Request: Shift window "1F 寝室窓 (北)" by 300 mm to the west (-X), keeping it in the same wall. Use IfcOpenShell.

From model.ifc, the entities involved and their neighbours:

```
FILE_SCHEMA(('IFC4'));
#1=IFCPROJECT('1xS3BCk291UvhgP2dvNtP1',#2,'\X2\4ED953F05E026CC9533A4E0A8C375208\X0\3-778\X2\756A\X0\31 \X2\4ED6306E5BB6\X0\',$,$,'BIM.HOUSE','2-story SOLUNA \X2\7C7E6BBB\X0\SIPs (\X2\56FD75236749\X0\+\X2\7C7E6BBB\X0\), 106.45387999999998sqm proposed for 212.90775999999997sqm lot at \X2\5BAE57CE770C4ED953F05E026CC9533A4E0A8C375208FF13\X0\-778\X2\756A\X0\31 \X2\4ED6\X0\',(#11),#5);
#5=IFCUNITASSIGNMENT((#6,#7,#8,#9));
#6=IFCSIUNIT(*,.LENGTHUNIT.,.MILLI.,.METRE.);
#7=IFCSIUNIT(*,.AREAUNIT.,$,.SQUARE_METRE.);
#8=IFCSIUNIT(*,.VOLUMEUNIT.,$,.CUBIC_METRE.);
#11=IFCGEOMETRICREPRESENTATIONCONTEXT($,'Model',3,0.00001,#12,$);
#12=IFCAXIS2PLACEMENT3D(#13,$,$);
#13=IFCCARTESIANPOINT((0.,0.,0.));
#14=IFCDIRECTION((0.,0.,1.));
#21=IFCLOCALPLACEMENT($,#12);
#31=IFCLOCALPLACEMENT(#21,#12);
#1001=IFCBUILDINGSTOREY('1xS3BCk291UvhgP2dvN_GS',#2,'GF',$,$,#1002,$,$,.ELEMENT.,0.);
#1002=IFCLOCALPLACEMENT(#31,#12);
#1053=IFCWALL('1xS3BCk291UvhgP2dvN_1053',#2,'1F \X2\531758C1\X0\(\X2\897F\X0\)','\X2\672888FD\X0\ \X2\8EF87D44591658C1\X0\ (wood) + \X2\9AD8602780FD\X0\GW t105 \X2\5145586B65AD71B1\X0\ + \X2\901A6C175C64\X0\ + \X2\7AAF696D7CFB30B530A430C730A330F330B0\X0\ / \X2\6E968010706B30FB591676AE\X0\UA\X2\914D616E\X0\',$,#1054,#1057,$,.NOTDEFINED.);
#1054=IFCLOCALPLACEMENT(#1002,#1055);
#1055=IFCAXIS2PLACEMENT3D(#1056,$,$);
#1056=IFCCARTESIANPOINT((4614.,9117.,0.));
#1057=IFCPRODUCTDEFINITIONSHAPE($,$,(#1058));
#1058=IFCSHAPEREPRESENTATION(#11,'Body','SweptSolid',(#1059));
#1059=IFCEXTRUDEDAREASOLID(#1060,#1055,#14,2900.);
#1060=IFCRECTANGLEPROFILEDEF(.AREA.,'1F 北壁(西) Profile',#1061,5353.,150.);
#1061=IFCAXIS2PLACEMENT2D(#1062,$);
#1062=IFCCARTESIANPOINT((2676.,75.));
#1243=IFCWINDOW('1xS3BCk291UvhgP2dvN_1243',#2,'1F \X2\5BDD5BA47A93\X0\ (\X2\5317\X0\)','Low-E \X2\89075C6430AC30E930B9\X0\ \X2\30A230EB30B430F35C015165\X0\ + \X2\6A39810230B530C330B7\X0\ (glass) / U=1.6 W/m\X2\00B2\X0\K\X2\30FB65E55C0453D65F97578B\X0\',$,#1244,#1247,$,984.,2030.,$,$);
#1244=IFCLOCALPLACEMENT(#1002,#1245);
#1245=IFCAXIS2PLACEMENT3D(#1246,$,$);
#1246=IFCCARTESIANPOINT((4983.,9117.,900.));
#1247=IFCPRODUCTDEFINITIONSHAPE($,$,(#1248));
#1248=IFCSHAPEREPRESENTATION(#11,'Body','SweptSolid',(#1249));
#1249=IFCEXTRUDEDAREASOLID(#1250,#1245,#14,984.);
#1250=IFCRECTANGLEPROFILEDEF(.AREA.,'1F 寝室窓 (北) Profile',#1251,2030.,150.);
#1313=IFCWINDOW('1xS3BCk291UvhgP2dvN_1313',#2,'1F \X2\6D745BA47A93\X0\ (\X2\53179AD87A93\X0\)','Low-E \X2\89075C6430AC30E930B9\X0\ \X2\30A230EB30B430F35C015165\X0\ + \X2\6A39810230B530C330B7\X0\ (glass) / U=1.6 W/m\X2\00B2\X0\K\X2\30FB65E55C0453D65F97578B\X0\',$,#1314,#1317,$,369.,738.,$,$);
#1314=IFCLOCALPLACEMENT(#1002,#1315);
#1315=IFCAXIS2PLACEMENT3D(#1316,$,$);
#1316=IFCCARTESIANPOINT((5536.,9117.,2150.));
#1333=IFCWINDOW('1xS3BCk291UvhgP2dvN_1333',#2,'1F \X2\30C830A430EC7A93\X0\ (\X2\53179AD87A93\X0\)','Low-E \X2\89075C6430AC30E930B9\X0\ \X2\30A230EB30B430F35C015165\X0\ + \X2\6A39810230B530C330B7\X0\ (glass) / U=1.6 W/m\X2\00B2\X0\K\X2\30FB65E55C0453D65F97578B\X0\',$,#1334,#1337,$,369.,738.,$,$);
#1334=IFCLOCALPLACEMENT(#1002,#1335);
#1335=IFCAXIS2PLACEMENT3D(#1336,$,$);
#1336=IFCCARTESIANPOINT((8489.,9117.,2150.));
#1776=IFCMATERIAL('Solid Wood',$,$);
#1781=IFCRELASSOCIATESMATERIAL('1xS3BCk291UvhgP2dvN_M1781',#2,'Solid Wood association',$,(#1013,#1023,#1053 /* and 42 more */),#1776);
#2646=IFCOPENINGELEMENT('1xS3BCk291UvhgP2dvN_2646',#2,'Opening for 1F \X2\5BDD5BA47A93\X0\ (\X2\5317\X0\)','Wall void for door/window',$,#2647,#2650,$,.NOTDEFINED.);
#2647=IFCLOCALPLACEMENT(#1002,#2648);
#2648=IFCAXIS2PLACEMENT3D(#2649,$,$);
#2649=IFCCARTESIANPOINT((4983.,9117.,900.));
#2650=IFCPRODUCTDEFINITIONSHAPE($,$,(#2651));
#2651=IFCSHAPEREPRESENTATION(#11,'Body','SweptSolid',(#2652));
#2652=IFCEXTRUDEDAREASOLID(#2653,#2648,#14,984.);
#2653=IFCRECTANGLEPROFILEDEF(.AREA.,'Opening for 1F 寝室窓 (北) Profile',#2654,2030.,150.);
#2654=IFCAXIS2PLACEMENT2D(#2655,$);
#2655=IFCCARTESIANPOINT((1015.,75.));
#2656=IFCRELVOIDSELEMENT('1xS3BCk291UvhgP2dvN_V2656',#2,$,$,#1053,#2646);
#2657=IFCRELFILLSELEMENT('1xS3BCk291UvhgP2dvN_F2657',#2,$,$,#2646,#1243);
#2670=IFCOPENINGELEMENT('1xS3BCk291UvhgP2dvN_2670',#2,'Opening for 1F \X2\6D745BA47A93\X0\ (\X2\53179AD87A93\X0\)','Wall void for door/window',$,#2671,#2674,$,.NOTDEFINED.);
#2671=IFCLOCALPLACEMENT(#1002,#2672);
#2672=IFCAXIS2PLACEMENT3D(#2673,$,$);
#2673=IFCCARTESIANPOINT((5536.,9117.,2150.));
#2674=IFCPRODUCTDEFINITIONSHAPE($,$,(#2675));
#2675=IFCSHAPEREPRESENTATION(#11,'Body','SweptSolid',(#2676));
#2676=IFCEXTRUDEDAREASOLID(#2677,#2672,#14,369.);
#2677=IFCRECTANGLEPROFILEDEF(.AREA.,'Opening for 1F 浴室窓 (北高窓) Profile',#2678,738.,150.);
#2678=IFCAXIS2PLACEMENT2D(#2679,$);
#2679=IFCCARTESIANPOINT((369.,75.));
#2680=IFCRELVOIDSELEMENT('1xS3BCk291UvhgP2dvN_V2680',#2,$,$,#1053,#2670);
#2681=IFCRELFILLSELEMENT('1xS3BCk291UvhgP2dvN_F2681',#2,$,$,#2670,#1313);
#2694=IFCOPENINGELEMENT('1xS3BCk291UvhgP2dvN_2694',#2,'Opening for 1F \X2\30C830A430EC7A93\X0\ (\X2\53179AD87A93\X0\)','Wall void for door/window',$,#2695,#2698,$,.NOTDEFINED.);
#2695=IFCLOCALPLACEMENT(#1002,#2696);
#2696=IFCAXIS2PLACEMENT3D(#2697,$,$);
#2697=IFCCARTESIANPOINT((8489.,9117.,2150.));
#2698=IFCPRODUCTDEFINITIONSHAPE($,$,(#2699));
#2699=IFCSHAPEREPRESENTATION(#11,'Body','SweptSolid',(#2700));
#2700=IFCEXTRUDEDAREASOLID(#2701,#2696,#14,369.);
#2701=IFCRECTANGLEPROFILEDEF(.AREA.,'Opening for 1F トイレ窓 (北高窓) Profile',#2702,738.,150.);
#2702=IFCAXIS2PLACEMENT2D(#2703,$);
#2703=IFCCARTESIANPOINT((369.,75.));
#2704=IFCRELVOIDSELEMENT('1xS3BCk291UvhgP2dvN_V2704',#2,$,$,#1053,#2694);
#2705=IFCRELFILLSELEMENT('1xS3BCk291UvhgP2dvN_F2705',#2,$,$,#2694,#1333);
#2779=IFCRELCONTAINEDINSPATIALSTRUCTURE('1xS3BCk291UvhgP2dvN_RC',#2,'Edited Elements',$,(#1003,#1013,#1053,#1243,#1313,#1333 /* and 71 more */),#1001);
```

```python
import ifcopenshell
import ifcopenshell.api.geometry
import ifcopenshell.util.placement
import ifcopenshell.util.unit

model = ifcopenshell.open("model.ifc")
unit_scale = ifcopenshell.util.unit.calculate_unit_scale(model)

window = model.by_id(1243)
opening = window.FillsVoids[0].RelatingOpeningElement
wall = opening.VoidsElements[0].RelatingBuildingElement

wall_matrix = ifcopenshell.util.placement.get_local_placement(wall.ObjectPlacement)
shift = wall_matrix[:3, 0] * -0.3 / unit_scale
before = ifcopenshell.util.placement.get_local_placement(window.ObjectPlacement)[:3, 3].copy()

# The window is not placed relative to its opening, so move both.
for product in (opening, window):
    matrix = ifcopenshell.util.placement.get_local_placement(product.ObjectPlacement)
    matrix[:3, 3] += shift
    ifcopenshell.api.geometry.edit_object_placement(model, product=product, matrix=matrix, is_si=False)

after = ifcopenshell.util.placement.get_local_placement(window.ObjectPlacement)[:3, 3]
print("window moved by", (after - before).round(3) + 0.0)

model.write("model-out.ifc")
```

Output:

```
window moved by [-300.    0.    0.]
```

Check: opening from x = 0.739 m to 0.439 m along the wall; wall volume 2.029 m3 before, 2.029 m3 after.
